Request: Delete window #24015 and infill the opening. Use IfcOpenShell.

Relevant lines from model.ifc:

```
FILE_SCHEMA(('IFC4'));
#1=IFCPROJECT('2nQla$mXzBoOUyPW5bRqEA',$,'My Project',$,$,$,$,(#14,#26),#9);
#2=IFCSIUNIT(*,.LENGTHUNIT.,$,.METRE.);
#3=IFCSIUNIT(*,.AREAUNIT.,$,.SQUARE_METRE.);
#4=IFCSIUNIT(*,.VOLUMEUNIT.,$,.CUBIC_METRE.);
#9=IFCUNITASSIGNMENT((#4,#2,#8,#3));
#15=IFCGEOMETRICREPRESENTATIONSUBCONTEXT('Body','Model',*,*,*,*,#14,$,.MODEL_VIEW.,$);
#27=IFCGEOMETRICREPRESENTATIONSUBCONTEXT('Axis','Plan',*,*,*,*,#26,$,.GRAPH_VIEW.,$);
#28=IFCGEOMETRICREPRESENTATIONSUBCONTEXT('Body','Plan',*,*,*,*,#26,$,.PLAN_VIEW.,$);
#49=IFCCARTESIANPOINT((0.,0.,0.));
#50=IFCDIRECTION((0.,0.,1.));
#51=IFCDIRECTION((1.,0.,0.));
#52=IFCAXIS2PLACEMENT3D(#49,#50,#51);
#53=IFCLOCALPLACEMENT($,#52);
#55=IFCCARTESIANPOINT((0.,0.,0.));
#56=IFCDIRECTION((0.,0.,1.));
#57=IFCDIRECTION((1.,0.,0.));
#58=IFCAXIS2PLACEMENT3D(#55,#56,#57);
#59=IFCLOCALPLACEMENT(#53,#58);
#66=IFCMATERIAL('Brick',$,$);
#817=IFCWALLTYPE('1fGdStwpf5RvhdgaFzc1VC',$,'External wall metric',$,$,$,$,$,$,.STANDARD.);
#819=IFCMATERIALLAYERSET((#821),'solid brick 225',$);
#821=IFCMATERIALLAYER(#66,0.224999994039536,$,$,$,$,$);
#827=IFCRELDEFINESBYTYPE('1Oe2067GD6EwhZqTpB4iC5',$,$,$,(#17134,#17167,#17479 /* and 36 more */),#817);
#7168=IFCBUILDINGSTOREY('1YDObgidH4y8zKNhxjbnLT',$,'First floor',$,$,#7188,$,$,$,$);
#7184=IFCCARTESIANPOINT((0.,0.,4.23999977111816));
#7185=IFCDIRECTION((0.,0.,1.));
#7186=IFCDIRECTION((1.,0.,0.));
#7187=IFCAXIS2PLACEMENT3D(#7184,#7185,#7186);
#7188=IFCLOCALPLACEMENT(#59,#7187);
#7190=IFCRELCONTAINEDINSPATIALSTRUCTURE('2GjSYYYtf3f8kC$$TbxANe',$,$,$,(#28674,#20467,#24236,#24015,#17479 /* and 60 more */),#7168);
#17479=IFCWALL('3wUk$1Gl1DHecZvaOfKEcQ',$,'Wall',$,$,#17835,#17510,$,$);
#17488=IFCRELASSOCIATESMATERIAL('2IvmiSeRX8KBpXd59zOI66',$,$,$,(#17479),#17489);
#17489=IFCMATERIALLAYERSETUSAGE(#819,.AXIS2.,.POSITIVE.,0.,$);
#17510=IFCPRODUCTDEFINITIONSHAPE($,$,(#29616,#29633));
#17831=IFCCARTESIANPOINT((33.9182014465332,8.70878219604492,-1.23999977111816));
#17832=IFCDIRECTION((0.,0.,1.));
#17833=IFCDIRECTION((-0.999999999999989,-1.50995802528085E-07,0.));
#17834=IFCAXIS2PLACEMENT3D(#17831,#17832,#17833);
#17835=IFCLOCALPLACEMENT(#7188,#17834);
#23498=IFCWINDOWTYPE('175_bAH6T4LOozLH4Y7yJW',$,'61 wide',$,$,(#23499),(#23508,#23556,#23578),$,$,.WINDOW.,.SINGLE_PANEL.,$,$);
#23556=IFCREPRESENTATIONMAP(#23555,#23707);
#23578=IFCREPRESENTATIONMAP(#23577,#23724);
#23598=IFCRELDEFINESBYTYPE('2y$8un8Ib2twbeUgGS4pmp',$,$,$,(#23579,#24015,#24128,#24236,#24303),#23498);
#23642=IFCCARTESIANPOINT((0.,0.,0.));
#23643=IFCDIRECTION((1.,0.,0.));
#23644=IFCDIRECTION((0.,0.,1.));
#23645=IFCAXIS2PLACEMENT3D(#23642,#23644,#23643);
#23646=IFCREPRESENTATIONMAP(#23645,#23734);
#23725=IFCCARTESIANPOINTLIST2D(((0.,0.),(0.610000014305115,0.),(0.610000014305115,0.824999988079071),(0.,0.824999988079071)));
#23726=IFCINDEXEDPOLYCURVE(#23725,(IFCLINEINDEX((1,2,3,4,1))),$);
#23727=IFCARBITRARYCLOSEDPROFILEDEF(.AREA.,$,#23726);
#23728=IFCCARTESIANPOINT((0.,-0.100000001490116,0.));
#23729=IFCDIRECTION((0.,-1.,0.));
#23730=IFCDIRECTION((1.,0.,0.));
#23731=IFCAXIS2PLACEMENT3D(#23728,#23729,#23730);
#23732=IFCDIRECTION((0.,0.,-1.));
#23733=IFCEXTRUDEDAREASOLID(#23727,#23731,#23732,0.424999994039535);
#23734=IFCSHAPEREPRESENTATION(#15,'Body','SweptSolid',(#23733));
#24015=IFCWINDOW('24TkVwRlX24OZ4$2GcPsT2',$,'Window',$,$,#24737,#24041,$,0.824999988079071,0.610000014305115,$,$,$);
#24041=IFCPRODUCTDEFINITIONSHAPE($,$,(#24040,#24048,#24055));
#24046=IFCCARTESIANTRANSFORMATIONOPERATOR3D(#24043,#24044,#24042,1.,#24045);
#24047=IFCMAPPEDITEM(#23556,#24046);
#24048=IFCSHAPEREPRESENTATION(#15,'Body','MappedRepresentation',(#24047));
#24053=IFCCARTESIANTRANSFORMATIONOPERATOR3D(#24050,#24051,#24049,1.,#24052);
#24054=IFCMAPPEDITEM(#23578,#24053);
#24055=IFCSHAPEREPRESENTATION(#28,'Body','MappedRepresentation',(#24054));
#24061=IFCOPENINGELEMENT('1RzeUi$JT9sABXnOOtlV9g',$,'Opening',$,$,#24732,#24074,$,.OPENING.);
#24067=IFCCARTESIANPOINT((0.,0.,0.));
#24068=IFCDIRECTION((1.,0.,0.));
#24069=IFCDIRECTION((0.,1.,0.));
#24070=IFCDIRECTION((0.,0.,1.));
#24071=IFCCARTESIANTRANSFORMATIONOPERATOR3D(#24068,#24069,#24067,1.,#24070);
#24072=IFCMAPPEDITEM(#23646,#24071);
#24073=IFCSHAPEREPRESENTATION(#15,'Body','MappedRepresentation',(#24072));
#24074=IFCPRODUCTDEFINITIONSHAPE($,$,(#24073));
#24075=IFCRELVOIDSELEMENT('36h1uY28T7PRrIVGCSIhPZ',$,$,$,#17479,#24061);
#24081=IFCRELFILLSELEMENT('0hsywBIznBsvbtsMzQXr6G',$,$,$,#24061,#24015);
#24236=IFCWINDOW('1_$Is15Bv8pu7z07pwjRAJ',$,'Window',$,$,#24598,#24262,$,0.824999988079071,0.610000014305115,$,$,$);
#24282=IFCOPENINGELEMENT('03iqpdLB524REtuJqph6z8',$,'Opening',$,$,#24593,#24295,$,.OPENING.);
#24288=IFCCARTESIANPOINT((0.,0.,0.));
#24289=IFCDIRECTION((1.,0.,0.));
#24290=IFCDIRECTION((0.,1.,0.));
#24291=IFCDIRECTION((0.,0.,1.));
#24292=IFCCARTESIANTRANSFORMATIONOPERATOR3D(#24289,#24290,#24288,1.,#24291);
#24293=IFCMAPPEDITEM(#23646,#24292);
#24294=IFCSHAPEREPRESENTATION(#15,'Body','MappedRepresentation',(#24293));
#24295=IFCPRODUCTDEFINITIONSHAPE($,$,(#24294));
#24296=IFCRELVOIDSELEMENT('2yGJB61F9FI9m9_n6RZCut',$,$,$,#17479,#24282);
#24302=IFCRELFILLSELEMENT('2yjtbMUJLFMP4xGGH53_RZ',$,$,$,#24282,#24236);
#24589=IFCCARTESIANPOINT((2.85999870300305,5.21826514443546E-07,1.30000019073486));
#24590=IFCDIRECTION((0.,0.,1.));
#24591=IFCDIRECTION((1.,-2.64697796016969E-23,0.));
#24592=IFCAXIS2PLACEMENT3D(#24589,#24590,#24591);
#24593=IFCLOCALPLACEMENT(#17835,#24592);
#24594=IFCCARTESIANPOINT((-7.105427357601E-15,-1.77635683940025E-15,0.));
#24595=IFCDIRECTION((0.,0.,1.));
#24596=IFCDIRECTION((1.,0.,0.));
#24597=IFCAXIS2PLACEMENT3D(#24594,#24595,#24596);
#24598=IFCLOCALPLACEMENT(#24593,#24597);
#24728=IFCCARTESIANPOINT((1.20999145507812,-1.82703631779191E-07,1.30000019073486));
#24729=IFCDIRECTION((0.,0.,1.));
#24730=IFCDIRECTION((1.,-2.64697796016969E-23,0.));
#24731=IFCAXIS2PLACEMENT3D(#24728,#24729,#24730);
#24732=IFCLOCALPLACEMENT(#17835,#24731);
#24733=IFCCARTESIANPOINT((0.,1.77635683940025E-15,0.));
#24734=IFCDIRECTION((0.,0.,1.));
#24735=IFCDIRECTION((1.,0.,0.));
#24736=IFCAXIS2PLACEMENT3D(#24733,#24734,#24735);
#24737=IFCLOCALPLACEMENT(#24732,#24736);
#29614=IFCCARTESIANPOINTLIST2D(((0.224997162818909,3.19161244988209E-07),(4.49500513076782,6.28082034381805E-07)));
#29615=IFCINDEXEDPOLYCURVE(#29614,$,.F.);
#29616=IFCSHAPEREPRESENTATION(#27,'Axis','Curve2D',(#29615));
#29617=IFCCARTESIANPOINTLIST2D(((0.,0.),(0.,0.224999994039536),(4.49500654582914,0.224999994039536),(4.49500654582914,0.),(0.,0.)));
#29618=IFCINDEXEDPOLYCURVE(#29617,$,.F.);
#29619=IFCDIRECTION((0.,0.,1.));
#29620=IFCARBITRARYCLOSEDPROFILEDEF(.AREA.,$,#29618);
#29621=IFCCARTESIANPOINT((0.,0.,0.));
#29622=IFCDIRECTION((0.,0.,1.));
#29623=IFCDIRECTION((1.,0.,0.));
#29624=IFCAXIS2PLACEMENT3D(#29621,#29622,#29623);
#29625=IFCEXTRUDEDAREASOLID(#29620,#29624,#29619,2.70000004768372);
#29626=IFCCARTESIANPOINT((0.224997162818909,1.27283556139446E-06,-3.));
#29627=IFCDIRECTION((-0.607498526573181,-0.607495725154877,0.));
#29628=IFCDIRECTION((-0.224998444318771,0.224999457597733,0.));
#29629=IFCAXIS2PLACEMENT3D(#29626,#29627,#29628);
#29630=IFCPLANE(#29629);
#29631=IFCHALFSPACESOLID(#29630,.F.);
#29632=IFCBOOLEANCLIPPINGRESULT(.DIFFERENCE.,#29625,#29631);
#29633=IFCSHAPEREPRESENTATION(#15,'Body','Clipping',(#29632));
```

```python
import ifcopenshell
import ifcopenshell.api.feature
import ifcopenshell.api.root
import ifcopenshell.geom
import ifcopenshell.util.shape

model = ifcopenshell.open("model.ifc")
settings = ifcopenshell.geom.settings()


def volume(element):
    """Net volume in cubic metres, openings subtracted."""
    shape = ifcopenshell.geom.create_shape(settings, element)
    return ifcopenshell.util.shape.get_volume(shape.geometry)


window = model.by_guid("24TkVwRlX24OZ4$2GcPsT2")
opening = window.FillsVoids[0].RelatingOpeningElement
wall = opening.VoidsElements[0].RelatingBuildingElement
before = volume(wall)

ifcopenshell.api.root.remove_product(model, product=window)
ifcopenshell.api.feature.remove_feature(model, feature=opening)

after = volume(wall)

print(f"wall volume {before:.3f} -> {after:.3f} m3")

model.write("model-out.ifc")
```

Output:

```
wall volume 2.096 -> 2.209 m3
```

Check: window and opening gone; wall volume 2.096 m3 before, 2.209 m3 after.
